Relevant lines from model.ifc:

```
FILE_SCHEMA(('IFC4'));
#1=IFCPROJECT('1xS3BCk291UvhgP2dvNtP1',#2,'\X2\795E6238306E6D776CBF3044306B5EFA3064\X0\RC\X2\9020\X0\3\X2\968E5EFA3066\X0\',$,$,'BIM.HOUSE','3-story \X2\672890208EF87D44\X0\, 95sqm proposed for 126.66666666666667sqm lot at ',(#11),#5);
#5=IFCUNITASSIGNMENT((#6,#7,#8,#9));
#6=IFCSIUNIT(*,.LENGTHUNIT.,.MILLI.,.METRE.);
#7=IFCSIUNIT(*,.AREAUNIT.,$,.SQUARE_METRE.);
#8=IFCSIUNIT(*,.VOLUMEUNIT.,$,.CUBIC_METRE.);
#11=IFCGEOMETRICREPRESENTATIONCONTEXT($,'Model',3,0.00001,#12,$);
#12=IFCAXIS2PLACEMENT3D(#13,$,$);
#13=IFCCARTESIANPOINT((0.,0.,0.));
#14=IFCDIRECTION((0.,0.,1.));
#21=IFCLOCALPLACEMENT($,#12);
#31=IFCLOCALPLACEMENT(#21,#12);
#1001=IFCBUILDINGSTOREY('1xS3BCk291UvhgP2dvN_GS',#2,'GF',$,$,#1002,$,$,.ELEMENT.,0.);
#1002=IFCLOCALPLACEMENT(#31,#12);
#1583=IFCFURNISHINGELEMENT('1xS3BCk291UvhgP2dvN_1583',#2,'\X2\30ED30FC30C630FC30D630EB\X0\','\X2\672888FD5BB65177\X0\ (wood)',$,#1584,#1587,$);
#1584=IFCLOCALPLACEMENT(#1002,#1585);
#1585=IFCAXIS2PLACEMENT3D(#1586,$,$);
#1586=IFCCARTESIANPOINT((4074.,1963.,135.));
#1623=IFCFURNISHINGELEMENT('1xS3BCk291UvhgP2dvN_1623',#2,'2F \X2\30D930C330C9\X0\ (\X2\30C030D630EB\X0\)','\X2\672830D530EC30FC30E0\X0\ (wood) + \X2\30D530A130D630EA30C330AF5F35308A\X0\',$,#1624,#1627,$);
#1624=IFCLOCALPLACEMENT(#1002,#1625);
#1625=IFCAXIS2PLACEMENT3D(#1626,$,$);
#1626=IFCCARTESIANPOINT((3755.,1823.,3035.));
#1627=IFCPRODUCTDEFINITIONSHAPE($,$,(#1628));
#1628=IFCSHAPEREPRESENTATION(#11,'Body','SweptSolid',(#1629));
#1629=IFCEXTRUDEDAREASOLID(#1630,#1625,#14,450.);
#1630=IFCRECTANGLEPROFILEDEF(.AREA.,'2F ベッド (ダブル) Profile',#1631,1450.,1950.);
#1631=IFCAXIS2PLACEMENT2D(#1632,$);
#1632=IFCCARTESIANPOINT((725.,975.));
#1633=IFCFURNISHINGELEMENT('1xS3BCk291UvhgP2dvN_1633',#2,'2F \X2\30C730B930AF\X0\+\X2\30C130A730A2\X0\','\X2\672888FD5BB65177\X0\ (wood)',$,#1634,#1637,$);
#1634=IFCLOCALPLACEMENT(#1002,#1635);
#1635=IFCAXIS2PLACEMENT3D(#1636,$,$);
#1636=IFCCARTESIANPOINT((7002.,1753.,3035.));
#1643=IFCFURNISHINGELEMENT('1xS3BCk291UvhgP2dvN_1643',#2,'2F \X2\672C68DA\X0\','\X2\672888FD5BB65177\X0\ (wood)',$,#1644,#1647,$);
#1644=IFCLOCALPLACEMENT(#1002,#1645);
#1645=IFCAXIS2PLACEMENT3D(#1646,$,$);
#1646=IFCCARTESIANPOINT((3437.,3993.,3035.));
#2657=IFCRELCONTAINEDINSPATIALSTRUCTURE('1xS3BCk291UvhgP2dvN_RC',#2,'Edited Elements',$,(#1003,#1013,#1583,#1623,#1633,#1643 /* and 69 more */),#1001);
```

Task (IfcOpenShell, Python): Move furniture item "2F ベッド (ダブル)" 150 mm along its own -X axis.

```python
import ifcopenshell
import ifcopenshell.api.geometry
import ifcopenshell.util.placement
import ifcopenshell.util.unit

model = ifcopenshell.open("model.ifc")
unit_scale = ifcopenshell.util.unit.calculate_unit_scale(model)

item = model.by_guid("1xS3BCk291UvhgP2dvN_1623")
matrix = ifcopenshell.util.placement.get_local_placement(item.ObjectPlacement)
matrix[:3, 3] -= matrix[:3, 0] * 0.15 / unit_scale
ifcopenshell.api.geometry.edit_object_placement(model, product=item, matrix=matrix, is_si=False)

print(ifcopenshell.util.placement.get_local_placement(item.ObjectPlacement).round(3) + 0.0)

model.write("model_edited.ifc")
```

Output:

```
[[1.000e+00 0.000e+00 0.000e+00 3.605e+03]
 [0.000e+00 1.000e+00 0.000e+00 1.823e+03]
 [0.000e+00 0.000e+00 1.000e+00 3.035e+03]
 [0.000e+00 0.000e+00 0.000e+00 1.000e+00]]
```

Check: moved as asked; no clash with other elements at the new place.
